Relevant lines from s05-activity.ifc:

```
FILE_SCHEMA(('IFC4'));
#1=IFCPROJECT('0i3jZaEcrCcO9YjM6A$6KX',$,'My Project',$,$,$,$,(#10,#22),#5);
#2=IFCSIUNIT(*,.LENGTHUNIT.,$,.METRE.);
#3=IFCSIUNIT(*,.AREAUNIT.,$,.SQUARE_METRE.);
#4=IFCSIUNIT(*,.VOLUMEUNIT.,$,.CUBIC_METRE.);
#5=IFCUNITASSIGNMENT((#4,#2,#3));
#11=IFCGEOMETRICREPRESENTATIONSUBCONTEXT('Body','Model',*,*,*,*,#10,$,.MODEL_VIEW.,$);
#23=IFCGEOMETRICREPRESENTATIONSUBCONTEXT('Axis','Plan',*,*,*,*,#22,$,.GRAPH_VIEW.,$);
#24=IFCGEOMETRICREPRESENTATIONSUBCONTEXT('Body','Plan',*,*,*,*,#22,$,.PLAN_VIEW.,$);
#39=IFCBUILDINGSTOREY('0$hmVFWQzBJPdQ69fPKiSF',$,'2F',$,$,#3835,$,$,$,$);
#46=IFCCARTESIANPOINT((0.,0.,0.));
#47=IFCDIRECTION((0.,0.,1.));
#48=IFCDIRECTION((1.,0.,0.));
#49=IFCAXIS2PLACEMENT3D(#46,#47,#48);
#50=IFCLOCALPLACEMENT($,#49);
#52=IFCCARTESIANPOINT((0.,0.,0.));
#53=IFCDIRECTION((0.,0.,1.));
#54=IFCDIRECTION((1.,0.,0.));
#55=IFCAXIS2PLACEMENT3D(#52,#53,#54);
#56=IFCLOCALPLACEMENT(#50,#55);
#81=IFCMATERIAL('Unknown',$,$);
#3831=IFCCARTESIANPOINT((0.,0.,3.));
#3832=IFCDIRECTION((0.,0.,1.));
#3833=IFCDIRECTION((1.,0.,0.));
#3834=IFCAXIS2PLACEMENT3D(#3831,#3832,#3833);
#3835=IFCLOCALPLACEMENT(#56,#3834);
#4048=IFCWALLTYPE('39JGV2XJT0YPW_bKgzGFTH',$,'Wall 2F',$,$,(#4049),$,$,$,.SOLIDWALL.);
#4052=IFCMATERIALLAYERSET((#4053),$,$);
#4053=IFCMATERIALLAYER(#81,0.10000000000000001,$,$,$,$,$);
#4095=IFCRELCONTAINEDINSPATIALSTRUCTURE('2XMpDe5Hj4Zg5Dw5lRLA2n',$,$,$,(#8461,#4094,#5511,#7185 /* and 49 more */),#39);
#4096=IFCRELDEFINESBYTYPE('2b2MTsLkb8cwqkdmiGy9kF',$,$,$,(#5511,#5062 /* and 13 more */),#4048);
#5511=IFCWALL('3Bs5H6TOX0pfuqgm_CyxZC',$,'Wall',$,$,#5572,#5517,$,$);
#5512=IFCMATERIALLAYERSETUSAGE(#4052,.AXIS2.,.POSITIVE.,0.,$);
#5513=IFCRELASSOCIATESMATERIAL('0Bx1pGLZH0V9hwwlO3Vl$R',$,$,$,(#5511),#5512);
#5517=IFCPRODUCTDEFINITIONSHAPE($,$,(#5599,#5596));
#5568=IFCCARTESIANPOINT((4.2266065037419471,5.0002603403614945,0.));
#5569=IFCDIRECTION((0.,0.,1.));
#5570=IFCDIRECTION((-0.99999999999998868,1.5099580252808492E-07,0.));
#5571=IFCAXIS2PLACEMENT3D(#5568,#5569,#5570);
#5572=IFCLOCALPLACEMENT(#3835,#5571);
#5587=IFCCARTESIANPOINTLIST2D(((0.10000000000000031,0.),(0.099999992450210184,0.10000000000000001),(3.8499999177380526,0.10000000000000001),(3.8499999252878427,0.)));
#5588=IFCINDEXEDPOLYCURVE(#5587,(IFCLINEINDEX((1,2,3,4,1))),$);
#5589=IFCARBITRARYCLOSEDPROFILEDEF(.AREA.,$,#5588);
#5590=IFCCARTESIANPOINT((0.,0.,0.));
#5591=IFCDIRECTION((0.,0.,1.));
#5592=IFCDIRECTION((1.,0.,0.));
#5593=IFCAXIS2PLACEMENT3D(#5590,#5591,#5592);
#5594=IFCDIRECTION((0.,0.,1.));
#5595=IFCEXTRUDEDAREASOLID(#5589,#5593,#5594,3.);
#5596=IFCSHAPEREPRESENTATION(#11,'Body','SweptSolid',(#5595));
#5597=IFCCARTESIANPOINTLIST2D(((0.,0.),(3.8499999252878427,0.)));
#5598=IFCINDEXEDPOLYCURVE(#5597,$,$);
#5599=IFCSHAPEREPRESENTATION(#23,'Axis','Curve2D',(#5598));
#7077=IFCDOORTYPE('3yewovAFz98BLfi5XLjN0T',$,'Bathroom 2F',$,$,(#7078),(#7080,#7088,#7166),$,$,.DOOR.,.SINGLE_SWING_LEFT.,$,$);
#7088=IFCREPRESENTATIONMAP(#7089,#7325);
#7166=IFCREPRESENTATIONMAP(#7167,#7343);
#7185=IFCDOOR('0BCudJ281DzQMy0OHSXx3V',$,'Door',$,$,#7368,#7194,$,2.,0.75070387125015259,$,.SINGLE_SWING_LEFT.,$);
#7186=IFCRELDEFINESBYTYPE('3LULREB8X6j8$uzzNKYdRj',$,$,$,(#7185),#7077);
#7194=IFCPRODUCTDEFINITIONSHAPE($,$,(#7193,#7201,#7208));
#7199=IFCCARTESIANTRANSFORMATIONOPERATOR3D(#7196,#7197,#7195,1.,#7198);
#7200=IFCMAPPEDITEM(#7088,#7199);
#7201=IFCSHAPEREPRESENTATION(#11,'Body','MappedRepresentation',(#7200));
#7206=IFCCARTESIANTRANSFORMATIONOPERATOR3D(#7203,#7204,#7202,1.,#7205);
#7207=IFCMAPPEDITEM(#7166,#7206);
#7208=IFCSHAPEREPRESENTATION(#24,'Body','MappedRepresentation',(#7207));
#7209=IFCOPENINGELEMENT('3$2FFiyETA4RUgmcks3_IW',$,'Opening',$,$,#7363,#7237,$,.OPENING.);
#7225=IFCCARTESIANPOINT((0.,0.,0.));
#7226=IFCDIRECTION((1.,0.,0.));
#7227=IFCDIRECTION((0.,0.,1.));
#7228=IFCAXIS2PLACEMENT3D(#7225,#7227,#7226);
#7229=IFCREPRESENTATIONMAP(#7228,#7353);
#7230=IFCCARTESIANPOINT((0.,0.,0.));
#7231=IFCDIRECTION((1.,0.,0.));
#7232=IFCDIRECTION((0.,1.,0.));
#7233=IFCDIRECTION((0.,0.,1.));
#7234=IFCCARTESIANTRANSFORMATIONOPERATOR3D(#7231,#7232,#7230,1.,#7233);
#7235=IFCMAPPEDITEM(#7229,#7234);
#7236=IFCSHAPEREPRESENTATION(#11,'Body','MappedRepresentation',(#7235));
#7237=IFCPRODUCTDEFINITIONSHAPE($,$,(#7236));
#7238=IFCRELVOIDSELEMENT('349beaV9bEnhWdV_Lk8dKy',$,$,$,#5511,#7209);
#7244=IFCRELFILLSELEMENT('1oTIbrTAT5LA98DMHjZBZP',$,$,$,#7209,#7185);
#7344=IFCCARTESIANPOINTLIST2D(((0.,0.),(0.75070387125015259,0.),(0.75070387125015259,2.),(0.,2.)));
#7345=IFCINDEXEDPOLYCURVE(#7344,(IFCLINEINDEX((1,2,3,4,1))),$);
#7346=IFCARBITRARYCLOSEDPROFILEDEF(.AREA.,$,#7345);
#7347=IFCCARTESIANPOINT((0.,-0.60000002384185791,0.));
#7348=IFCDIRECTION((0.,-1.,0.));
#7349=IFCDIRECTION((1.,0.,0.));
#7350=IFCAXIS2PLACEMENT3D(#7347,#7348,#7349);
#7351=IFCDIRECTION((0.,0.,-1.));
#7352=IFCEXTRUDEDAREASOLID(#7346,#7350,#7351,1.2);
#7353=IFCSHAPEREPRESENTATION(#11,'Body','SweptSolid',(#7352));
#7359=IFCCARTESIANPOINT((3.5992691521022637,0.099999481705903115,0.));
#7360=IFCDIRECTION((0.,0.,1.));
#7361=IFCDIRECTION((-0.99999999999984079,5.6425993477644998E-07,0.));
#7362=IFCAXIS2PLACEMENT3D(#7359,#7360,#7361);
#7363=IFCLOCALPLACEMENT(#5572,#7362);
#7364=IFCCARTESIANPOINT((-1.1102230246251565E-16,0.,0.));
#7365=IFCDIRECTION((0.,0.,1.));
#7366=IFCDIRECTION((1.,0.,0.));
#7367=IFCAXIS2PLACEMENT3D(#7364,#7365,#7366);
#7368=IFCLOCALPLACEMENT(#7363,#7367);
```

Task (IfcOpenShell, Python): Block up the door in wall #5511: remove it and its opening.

```python
import ifcopenshell
import ifcopenshell.api.feature
import ifcopenshell.api.root
import ifcopenshell.geom
import ifcopenshell.util.shape

model = ifcopenshell.open("s05-activity.ifc")
settings = ifcopenshell.geom.settings()


def volume(element):
    """Net volume in cubic metres, openings subtracted."""
    shape = ifcopenshell.geom.create_shape(settings, element)
    return ifcopenshell.util.shape.get_volume(shape.geometry)


door = model.by_guid("0BCudJ281DzQMy0OHSXx3V")
opening = door.FillsVoids[0].RelatingOpeningElement
wall = opening.VoidsElements[0].RelatingBuildingElement
before = volume(wall)

ifcopenshell.api.root.remove_product(model, product=door)
ifcopenshell.api.feature.remove_feature(model, feature=opening)

after = volume(wall)

print(f"wall volume {before:.3f} -> {after:.3f} m3")

model.write("s05-activity_rev.ifc")
```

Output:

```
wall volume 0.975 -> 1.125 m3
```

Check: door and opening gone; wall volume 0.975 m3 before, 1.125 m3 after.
